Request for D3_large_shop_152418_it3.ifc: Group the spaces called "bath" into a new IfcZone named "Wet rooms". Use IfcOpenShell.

First a look at what the model holds.

```python
import ifcopenshell

model = ifcopenshell.open("D3_large_shop_152418_it3.ifc")
print(model.schema)
seen = {}
for space in model.by_type("IfcSpace"):
    seen[space.LongName] = seen.get(space.LongName, 0) + 1
for name, count in sorted(seen.items(), key=str):
    print(count, "x", name)
print("zones:", [z.Name for z in model.by_type("IfcZone")][:20])
```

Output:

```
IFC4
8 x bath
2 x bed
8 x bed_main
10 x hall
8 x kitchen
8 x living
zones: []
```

```python
import ifcopenshell
import ifcopenshell.api.group
import ifcopenshell.api.root

model = ifcopenshell.open("D3_large_shop_152418_it3.ifc")

names = {"bath"}
spaces = [s for s in model.by_type("IfcSpace") if s.LongName in names]

zone = ifcopenshell.api.root.create_entity(model, ifc_class="IfcZone", name="Wet rooms")
ifcopenshell.api.group.assign_group(model, products=spaces, group=zone)
print(len(spaces), "spaces in", zone.Name)

model.write("D3_large_shop_152418_it3-out.ifc")
```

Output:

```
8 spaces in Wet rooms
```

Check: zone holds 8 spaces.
